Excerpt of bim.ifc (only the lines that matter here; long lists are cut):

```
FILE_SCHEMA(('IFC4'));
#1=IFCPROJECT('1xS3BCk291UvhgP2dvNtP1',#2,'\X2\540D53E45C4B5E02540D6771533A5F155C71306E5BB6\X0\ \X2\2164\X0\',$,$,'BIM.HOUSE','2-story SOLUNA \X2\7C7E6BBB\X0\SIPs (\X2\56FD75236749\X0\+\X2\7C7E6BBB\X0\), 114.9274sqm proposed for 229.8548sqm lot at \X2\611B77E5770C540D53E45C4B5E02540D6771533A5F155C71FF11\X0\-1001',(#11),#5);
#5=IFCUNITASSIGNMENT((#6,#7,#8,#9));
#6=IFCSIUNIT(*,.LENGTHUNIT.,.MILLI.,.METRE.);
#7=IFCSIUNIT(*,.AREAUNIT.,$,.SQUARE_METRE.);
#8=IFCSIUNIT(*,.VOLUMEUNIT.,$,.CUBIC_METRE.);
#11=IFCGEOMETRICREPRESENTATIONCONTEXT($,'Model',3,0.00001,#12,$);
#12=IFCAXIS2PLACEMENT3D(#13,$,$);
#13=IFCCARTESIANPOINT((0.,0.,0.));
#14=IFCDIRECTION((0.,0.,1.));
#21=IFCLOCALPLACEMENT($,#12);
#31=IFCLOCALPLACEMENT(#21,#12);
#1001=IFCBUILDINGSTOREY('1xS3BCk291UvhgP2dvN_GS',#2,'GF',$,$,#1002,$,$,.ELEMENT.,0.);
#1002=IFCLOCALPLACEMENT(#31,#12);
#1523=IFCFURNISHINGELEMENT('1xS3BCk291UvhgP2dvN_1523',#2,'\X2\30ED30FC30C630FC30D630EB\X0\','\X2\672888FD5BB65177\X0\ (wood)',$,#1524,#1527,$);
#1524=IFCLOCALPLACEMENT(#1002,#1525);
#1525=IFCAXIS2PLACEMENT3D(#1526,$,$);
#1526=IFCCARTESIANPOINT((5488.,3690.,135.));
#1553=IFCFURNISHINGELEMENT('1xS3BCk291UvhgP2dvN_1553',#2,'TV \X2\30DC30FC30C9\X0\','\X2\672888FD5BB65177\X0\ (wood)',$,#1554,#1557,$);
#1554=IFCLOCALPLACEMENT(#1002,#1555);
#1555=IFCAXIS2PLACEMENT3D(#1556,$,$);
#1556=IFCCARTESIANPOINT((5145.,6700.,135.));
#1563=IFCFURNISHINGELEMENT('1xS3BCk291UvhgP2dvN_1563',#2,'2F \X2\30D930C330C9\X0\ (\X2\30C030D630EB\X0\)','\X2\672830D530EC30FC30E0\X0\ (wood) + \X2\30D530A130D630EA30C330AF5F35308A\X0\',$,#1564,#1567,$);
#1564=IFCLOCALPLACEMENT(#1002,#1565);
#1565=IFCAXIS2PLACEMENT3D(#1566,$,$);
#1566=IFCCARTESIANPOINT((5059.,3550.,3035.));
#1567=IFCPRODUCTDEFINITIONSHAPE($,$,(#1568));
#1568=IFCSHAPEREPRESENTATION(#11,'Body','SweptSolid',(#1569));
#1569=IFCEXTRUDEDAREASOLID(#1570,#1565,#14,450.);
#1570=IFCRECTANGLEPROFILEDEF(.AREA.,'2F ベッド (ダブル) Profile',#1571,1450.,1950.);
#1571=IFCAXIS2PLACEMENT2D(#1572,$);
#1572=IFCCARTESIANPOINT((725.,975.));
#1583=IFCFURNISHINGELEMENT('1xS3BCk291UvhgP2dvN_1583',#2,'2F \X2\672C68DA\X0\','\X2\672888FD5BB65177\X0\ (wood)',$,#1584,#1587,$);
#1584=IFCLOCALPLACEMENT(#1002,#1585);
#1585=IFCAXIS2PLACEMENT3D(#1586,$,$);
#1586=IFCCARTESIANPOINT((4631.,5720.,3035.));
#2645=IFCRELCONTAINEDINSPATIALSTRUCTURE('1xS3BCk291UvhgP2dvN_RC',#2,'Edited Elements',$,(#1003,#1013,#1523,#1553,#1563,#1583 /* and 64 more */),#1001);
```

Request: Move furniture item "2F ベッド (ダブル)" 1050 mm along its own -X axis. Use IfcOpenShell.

```python
import ifcopenshell
import ifcopenshell.api.geometry
import ifcopenshell.util.placement
import ifcopenshell.util.unit

model = ifcopenshell.open("bim.ifc")
unit_scale = ifcopenshell.util.unit.calculate_unit_scale(model)

item = model.by_guid("1xS3BCk291UvhgP2dvN_1563")
matrix = ifcopenshell.util.placement.get_local_placement(item.ObjectPlacement)
matrix[:3, 3] -= matrix[:3, 0] * 1.05 / unit_scale
ifcopenshell.api.geometry.edit_object_placement(model, product=item, matrix=matrix, is_si=False)

print(ifcopenshell.util.placement.get_local_placement(item.ObjectPlacement).round(3) + 0.0)

model.write("bim_v2.ifc")
```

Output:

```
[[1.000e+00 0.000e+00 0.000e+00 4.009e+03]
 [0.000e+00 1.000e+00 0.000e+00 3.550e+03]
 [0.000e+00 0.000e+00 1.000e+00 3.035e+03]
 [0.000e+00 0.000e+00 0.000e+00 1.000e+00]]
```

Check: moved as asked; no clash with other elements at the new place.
